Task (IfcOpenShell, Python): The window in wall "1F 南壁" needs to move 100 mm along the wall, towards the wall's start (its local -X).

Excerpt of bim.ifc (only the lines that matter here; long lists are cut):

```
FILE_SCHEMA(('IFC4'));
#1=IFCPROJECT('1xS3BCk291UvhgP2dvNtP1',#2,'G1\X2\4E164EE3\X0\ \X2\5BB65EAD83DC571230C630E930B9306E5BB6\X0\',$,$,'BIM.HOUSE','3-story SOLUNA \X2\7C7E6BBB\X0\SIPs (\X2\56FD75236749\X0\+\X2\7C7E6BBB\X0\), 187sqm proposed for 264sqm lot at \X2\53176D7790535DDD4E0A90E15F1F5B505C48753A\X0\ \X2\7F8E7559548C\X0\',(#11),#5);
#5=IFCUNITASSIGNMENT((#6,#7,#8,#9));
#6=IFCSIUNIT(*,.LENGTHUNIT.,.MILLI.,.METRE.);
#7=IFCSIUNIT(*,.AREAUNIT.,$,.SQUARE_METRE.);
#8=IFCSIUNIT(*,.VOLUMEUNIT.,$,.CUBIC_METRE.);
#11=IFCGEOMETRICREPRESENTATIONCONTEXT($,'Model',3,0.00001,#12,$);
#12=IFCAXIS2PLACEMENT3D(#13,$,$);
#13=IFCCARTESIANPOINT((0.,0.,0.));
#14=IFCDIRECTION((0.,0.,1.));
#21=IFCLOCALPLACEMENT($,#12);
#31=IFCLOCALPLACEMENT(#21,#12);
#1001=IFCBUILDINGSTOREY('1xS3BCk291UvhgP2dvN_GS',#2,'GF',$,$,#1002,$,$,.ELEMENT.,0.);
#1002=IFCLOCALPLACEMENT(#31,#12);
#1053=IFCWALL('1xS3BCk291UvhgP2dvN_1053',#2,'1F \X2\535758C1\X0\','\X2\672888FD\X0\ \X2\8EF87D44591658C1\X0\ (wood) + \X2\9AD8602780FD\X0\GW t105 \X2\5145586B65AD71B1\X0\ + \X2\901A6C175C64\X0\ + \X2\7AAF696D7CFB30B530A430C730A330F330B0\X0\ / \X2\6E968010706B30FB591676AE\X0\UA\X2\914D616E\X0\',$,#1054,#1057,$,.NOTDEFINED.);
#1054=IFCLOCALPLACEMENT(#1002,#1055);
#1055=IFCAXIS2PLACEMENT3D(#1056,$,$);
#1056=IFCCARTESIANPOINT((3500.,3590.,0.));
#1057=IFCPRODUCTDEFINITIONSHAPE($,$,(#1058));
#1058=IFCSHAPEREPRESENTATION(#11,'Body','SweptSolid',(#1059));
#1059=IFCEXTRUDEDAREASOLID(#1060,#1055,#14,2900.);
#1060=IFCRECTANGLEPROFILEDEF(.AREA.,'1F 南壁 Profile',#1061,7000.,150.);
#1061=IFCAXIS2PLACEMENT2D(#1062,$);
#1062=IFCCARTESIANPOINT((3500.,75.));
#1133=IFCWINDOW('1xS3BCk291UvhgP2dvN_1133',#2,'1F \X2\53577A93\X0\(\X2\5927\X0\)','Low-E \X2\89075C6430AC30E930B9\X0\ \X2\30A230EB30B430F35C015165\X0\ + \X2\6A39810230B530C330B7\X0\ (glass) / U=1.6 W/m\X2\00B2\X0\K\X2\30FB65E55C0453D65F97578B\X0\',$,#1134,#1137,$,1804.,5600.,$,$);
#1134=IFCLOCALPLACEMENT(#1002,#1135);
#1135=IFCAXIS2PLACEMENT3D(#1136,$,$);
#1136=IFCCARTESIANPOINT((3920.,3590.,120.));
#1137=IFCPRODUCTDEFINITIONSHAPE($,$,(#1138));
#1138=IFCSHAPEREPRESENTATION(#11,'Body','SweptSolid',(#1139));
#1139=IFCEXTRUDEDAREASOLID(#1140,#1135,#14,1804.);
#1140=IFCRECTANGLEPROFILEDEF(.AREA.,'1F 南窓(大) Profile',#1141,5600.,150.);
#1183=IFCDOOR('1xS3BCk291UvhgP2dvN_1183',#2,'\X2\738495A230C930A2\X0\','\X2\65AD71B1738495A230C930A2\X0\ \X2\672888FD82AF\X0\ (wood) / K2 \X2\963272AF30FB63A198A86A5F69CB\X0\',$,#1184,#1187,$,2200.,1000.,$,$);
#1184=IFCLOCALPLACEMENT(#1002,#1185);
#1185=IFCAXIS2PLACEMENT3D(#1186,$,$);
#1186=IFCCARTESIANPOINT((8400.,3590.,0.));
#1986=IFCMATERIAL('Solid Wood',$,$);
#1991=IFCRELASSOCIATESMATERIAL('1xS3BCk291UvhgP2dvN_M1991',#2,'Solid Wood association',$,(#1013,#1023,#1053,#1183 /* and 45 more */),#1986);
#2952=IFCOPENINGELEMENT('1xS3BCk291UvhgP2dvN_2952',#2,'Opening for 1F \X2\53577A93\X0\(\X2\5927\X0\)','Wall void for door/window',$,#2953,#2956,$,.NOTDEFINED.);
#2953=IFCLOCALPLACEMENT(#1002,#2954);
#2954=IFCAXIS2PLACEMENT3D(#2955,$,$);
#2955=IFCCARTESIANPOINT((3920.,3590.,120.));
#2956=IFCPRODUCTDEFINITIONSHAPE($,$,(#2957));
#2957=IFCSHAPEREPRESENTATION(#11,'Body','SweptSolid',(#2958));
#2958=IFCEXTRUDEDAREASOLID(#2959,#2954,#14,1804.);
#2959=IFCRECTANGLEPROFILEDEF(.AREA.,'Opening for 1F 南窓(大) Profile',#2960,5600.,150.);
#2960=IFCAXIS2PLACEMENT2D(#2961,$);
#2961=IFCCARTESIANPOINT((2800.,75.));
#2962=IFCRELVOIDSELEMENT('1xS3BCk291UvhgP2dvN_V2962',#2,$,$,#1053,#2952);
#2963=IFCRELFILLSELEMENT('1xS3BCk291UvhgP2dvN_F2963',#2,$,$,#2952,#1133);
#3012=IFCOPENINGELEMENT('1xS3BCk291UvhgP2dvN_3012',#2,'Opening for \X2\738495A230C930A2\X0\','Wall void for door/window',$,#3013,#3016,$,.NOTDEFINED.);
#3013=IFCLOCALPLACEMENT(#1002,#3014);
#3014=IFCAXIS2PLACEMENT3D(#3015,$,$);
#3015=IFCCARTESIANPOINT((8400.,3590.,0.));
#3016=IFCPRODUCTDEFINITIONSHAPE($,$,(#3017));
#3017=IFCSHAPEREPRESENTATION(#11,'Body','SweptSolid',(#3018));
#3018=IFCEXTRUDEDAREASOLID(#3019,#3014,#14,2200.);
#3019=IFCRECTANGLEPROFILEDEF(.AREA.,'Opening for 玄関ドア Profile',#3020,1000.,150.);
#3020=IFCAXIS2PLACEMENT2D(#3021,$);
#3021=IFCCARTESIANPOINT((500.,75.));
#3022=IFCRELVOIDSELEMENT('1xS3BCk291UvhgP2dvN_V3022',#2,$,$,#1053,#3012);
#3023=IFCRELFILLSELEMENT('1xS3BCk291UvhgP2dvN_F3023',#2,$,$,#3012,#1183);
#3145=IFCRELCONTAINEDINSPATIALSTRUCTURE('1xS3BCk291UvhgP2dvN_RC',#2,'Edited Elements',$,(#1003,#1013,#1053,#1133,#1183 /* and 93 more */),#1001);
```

```python
import ifcopenshell
import ifcopenshell.api.geometry
import ifcopenshell.util.placement
import ifcopenshell.util.unit

model = ifcopenshell.open("bim.ifc")
unit_scale = ifcopenshell.util.unit.calculate_unit_scale(model)

window = model.by_guid("1xS3BCk291UvhgP2dvN_1133")
opening = window.FillsVoids[0].RelatingOpeningElement
wall = opening.VoidsElements[0].RelatingBuildingElement

wall_matrix = ifcopenshell.util.placement.get_local_placement(wall.ObjectPlacement)
shift = wall_matrix[:3, 0] * -0.1 / unit_scale
before = ifcopenshell.util.placement.get_local_placement(window.ObjectPlacement)[:3, 3].copy()

# The window is not placed relative to its opening, so move both.
for product in (opening, window):
    matrix = ifcopenshell.util.placement.get_local_placement(product.ObjectPlacement)
    matrix[:3, 3] += shift
    ifcopenshell.api.geometry.edit_object_placement(model, product=product, matrix=matrix, is_si=False)

after = ifcopenshell.util.placement.get_local_placement(window.ObjectPlacement)[:3, 3]
print("window moved by", (after - before).round(3) + 0.0)

model.write("bim-out.ifc")
```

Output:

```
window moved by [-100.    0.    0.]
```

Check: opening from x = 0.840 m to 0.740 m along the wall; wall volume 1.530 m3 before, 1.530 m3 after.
